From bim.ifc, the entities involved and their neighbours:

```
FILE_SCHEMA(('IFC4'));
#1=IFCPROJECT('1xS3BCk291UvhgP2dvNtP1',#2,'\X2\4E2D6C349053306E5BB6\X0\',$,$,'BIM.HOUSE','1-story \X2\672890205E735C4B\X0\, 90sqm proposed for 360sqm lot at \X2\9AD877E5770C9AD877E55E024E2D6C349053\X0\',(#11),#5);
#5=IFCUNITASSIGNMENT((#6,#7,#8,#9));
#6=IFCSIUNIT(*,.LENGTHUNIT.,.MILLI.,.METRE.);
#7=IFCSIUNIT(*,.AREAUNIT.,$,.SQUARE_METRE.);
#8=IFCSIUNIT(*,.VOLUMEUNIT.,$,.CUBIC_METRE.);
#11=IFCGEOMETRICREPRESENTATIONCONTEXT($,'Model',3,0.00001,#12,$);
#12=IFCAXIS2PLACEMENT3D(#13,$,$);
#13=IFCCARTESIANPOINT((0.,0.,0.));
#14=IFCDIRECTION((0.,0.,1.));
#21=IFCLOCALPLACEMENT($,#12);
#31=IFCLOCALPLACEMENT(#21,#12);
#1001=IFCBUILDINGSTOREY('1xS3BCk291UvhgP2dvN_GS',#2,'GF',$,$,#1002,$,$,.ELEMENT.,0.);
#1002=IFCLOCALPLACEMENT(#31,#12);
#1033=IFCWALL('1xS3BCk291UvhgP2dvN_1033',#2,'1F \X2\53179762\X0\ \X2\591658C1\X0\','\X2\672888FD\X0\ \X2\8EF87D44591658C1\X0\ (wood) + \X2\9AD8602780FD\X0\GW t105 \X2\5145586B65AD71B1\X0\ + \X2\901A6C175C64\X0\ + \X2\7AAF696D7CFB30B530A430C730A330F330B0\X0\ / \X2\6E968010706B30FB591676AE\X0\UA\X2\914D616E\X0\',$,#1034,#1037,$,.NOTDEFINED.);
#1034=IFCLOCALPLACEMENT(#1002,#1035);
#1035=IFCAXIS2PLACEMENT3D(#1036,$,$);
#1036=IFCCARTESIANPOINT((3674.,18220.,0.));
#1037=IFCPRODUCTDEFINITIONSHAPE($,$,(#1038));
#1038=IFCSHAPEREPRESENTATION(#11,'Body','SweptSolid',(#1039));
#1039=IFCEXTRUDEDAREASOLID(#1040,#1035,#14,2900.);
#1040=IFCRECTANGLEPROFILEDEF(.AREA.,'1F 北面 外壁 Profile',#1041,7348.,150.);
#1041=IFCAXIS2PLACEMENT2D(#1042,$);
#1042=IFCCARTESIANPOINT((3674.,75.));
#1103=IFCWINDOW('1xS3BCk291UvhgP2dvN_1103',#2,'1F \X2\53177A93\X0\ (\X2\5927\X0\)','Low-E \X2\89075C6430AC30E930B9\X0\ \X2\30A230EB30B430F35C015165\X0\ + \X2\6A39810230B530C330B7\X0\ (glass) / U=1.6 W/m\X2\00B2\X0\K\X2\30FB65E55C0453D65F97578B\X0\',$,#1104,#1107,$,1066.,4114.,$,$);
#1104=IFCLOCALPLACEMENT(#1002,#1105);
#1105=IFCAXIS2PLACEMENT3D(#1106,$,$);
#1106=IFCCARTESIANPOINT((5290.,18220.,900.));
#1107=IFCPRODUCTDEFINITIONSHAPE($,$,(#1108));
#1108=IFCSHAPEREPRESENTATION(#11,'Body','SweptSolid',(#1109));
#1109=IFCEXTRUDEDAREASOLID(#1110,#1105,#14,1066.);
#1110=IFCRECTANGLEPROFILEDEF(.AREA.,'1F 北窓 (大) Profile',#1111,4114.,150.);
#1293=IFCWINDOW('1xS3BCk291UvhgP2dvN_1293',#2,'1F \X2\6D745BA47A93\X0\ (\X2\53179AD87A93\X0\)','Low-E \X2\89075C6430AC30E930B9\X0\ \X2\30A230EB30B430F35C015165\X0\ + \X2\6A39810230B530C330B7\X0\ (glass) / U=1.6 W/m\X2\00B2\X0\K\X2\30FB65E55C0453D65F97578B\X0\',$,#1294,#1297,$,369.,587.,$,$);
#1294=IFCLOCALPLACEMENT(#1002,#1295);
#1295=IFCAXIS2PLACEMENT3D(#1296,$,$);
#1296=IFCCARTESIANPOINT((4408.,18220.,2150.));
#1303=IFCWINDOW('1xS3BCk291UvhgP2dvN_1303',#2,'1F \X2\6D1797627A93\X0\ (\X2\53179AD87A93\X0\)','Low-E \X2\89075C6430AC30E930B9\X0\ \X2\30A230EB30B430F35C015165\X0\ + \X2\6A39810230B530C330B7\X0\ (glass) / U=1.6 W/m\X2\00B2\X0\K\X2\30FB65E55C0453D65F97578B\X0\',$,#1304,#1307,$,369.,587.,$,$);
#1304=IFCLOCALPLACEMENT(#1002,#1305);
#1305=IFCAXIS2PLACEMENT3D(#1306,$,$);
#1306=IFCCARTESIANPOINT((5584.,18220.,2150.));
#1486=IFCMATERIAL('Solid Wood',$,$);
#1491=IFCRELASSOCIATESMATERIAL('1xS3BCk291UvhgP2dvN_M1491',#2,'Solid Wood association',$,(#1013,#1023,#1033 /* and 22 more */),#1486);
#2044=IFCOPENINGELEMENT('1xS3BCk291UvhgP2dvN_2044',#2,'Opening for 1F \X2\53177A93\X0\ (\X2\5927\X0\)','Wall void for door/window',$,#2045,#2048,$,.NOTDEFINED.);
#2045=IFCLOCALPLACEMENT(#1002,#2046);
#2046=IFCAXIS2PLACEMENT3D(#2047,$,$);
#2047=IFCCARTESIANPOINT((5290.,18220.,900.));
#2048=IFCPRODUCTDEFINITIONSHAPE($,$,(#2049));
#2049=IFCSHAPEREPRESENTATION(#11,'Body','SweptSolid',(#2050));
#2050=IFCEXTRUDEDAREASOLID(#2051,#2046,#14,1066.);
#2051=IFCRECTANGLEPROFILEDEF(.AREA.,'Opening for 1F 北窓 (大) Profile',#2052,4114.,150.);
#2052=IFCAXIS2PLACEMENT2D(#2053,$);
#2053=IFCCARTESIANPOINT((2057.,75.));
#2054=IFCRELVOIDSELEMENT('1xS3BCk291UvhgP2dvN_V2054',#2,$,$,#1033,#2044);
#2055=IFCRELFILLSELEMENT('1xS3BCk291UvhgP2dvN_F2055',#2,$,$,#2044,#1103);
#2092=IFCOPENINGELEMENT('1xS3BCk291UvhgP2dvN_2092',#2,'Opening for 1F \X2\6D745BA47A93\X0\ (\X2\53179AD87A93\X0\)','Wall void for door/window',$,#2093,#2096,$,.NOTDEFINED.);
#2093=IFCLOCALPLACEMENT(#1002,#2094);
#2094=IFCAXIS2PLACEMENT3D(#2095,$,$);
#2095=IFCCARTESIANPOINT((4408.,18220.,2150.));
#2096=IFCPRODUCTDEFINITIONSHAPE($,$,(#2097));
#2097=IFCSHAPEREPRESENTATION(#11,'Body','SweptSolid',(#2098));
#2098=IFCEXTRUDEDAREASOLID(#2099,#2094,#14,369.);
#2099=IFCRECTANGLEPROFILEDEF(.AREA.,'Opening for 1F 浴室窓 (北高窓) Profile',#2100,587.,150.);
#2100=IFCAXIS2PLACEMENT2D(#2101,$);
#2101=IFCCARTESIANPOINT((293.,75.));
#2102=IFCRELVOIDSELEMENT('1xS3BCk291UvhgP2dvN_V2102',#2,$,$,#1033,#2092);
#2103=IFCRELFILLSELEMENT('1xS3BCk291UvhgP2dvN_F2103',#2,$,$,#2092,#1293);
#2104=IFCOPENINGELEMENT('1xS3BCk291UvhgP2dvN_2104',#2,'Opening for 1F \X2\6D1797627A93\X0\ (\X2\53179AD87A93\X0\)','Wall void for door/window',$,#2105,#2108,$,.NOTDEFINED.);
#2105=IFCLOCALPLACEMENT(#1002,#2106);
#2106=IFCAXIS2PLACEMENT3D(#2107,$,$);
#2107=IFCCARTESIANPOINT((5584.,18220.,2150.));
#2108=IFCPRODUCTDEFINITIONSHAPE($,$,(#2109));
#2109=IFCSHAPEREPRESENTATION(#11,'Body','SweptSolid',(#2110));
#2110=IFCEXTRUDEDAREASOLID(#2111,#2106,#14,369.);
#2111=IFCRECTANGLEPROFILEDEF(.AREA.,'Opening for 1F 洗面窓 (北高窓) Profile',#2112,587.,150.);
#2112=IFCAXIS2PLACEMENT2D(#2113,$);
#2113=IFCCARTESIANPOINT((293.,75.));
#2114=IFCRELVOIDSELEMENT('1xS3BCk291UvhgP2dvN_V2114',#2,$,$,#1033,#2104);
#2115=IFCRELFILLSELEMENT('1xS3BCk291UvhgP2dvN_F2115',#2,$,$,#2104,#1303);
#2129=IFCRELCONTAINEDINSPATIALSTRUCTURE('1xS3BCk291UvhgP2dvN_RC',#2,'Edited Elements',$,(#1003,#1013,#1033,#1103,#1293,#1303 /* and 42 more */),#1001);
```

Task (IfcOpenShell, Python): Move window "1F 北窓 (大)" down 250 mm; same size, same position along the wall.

```python
import numpy as np
import ifcopenshell
import ifcopenshell.api.geometry
import ifcopenshell.util.placement
import ifcopenshell.util.unit

model = ifcopenshell.open("bim.ifc")
unit_scale = ifcopenshell.util.unit.calculate_unit_scale(model)

window = model.by_guid("1xS3BCk291UvhgP2dvN_1103")
opening = window.FillsVoids[0].RelatingOpeningElement
dz = -0.25 / unit_scale

shift = np.array([0.0, 0.0, dz])
# The window is not placed relative to its opening, so move both.
for product in (opening, window):
    matrix = ifcopenshell.util.placement.get_local_placement(product.ObjectPlacement)
    matrix[:3, 3] += shift
    ifcopenshell.api.geometry.edit_object_placement(model, product=product, matrix=matrix, is_si=False)

print(f"moved by {dz * unit_scale:+.3f} m")

model.write("bim_v2.ifc")
```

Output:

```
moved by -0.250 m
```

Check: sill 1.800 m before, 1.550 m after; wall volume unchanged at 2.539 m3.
